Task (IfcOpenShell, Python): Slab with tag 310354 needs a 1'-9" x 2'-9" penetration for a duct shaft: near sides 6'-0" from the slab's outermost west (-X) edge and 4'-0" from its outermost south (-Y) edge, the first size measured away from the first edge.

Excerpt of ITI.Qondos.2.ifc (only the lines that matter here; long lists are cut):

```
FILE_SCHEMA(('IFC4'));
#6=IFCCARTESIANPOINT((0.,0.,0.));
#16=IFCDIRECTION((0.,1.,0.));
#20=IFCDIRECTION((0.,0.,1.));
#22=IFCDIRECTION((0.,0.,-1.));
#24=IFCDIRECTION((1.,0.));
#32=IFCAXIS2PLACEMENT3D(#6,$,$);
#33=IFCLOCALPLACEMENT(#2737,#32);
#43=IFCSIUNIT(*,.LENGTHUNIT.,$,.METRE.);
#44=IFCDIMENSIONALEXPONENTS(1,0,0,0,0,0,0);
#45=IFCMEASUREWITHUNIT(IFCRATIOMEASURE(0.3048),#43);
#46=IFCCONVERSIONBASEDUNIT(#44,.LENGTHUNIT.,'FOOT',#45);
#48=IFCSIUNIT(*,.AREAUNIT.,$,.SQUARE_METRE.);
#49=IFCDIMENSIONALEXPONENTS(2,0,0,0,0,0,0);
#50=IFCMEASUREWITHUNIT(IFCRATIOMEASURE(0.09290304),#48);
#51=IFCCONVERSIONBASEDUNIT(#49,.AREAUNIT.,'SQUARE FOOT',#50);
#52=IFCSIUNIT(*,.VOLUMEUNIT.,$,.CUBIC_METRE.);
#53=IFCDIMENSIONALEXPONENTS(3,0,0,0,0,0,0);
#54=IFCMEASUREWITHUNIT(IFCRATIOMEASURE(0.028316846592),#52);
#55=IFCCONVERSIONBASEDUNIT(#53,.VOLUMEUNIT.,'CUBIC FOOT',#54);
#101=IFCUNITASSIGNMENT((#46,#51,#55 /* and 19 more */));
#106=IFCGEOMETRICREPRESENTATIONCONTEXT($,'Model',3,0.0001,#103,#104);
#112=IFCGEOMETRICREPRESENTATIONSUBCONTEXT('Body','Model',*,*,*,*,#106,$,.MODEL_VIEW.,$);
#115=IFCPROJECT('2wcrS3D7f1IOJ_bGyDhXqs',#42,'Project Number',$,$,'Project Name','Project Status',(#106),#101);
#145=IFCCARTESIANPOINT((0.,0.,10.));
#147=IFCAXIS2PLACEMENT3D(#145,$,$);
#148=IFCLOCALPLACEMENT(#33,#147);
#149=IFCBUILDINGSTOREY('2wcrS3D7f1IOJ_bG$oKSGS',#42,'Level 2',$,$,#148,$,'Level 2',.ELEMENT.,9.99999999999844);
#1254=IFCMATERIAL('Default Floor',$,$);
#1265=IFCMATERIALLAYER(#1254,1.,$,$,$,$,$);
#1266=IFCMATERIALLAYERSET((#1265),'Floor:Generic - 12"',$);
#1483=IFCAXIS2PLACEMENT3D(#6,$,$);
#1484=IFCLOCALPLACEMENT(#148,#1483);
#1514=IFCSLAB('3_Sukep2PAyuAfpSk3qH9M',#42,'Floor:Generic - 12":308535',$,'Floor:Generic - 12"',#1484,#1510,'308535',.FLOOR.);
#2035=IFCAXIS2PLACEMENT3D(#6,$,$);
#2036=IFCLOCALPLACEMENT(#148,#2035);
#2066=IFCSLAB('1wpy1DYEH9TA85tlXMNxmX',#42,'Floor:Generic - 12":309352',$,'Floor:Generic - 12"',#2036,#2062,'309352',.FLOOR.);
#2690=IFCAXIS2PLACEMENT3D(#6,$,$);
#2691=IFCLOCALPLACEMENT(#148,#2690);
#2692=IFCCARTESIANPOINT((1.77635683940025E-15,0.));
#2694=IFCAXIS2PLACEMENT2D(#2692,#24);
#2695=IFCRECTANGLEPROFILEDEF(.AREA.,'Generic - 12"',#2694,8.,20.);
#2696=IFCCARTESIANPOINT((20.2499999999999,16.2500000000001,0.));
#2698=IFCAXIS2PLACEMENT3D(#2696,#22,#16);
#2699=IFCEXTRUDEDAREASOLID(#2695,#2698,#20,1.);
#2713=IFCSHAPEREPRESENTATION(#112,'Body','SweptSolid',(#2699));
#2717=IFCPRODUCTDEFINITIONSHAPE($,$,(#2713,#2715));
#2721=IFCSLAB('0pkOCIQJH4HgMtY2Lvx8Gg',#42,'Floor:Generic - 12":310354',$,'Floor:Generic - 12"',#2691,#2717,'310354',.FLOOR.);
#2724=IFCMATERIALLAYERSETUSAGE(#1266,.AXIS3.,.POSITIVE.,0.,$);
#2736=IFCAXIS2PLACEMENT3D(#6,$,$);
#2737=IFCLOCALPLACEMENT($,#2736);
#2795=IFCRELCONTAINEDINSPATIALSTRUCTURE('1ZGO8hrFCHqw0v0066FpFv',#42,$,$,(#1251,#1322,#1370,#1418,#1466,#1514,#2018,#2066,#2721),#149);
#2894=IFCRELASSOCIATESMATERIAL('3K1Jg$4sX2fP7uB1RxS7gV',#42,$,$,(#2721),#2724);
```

```python
import numpy as np
import ifcopenshell
import ifcopenshell.api.feature
import ifcopenshell.api.geometry
import ifcopenshell.api.root
import ifcopenshell.geom
import ifcopenshell.util.placement
import ifcopenshell.util.representation
import ifcopenshell.util.shape
import ifcopenshell.util.unit

model = ifcopenshell.open("ITI.Qondos.2.ifc")
unit_scale = ifcopenshell.util.unit.calculate_unit_scale(model)
settings = ifcopenshell.geom.settings()


def volume(element):
    """Net volume in cubic metres, openings subtracted."""
    shape = ifcopenshell.geom.create_shape(settings, element)
    return ifcopenshell.util.shape.get_volume(shape.geometry)


slab = model.by_guid("0pkOCIQJH4HgMtY2Lvx8Gg")
before = volume(slab)

# Extent in the slab's own axes, in metres. The edges named are its -X and -Y sides.
slab_shape = ifcopenshell.geom.create_shape(settings, slab)
vertices = ifcopenshell.util.shape.get_vertices(slab_shape.geometry)
x_min, y_min, bottom = vertices.min(axis=0)
top = vertices[:, 2].max()

opening = ifcopenshell.api.root.create_entity(model, ifc_class="IfcOpeningElement", name="Duct shaft opening", predefined_type="OPENING")
context = ifcopenshell.util.representation.get_context(model, "Model", "Body", "MODEL_VIEW")
width, depth = 0.5334, 0.8382
outline = [(0.0, 0.0), (width, 0.0), (width, depth), (0.0, depth), (0.0, 0.0)]
# Overshoot both faces by 50 mm so the cut is clean.
shape = ifcopenshell.api.geometry.add_slab_representation(
    model, context=context, depth=top - bottom + 0.1, polyline=outline
)
ifcopenshell.api.geometry.assign_representation(model, product=opening, representation=shape)

matrix = ifcopenshell.util.placement.get_local_placement(slab.ObjectPlacement)
matrix[:, 3] = matrix @ np.append(np.array([x_min + 1.8288, y_min + 1.2192, bottom - 0.05]) / unit_scale, 1.0)
ifcopenshell.api.geometry.edit_object_placement(model, product=opening, matrix=matrix, is_si=False)
ifcopenshell.api.feature.add_feature(model, feature=opening, element=slab)

after = volume(slab)

print(f"slab volume {before:.3f} -> {after:.3f} m3")

model.write("ITI.Qondos.2_rev.ifc")
```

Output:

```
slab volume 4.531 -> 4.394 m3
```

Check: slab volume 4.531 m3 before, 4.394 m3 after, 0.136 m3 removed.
